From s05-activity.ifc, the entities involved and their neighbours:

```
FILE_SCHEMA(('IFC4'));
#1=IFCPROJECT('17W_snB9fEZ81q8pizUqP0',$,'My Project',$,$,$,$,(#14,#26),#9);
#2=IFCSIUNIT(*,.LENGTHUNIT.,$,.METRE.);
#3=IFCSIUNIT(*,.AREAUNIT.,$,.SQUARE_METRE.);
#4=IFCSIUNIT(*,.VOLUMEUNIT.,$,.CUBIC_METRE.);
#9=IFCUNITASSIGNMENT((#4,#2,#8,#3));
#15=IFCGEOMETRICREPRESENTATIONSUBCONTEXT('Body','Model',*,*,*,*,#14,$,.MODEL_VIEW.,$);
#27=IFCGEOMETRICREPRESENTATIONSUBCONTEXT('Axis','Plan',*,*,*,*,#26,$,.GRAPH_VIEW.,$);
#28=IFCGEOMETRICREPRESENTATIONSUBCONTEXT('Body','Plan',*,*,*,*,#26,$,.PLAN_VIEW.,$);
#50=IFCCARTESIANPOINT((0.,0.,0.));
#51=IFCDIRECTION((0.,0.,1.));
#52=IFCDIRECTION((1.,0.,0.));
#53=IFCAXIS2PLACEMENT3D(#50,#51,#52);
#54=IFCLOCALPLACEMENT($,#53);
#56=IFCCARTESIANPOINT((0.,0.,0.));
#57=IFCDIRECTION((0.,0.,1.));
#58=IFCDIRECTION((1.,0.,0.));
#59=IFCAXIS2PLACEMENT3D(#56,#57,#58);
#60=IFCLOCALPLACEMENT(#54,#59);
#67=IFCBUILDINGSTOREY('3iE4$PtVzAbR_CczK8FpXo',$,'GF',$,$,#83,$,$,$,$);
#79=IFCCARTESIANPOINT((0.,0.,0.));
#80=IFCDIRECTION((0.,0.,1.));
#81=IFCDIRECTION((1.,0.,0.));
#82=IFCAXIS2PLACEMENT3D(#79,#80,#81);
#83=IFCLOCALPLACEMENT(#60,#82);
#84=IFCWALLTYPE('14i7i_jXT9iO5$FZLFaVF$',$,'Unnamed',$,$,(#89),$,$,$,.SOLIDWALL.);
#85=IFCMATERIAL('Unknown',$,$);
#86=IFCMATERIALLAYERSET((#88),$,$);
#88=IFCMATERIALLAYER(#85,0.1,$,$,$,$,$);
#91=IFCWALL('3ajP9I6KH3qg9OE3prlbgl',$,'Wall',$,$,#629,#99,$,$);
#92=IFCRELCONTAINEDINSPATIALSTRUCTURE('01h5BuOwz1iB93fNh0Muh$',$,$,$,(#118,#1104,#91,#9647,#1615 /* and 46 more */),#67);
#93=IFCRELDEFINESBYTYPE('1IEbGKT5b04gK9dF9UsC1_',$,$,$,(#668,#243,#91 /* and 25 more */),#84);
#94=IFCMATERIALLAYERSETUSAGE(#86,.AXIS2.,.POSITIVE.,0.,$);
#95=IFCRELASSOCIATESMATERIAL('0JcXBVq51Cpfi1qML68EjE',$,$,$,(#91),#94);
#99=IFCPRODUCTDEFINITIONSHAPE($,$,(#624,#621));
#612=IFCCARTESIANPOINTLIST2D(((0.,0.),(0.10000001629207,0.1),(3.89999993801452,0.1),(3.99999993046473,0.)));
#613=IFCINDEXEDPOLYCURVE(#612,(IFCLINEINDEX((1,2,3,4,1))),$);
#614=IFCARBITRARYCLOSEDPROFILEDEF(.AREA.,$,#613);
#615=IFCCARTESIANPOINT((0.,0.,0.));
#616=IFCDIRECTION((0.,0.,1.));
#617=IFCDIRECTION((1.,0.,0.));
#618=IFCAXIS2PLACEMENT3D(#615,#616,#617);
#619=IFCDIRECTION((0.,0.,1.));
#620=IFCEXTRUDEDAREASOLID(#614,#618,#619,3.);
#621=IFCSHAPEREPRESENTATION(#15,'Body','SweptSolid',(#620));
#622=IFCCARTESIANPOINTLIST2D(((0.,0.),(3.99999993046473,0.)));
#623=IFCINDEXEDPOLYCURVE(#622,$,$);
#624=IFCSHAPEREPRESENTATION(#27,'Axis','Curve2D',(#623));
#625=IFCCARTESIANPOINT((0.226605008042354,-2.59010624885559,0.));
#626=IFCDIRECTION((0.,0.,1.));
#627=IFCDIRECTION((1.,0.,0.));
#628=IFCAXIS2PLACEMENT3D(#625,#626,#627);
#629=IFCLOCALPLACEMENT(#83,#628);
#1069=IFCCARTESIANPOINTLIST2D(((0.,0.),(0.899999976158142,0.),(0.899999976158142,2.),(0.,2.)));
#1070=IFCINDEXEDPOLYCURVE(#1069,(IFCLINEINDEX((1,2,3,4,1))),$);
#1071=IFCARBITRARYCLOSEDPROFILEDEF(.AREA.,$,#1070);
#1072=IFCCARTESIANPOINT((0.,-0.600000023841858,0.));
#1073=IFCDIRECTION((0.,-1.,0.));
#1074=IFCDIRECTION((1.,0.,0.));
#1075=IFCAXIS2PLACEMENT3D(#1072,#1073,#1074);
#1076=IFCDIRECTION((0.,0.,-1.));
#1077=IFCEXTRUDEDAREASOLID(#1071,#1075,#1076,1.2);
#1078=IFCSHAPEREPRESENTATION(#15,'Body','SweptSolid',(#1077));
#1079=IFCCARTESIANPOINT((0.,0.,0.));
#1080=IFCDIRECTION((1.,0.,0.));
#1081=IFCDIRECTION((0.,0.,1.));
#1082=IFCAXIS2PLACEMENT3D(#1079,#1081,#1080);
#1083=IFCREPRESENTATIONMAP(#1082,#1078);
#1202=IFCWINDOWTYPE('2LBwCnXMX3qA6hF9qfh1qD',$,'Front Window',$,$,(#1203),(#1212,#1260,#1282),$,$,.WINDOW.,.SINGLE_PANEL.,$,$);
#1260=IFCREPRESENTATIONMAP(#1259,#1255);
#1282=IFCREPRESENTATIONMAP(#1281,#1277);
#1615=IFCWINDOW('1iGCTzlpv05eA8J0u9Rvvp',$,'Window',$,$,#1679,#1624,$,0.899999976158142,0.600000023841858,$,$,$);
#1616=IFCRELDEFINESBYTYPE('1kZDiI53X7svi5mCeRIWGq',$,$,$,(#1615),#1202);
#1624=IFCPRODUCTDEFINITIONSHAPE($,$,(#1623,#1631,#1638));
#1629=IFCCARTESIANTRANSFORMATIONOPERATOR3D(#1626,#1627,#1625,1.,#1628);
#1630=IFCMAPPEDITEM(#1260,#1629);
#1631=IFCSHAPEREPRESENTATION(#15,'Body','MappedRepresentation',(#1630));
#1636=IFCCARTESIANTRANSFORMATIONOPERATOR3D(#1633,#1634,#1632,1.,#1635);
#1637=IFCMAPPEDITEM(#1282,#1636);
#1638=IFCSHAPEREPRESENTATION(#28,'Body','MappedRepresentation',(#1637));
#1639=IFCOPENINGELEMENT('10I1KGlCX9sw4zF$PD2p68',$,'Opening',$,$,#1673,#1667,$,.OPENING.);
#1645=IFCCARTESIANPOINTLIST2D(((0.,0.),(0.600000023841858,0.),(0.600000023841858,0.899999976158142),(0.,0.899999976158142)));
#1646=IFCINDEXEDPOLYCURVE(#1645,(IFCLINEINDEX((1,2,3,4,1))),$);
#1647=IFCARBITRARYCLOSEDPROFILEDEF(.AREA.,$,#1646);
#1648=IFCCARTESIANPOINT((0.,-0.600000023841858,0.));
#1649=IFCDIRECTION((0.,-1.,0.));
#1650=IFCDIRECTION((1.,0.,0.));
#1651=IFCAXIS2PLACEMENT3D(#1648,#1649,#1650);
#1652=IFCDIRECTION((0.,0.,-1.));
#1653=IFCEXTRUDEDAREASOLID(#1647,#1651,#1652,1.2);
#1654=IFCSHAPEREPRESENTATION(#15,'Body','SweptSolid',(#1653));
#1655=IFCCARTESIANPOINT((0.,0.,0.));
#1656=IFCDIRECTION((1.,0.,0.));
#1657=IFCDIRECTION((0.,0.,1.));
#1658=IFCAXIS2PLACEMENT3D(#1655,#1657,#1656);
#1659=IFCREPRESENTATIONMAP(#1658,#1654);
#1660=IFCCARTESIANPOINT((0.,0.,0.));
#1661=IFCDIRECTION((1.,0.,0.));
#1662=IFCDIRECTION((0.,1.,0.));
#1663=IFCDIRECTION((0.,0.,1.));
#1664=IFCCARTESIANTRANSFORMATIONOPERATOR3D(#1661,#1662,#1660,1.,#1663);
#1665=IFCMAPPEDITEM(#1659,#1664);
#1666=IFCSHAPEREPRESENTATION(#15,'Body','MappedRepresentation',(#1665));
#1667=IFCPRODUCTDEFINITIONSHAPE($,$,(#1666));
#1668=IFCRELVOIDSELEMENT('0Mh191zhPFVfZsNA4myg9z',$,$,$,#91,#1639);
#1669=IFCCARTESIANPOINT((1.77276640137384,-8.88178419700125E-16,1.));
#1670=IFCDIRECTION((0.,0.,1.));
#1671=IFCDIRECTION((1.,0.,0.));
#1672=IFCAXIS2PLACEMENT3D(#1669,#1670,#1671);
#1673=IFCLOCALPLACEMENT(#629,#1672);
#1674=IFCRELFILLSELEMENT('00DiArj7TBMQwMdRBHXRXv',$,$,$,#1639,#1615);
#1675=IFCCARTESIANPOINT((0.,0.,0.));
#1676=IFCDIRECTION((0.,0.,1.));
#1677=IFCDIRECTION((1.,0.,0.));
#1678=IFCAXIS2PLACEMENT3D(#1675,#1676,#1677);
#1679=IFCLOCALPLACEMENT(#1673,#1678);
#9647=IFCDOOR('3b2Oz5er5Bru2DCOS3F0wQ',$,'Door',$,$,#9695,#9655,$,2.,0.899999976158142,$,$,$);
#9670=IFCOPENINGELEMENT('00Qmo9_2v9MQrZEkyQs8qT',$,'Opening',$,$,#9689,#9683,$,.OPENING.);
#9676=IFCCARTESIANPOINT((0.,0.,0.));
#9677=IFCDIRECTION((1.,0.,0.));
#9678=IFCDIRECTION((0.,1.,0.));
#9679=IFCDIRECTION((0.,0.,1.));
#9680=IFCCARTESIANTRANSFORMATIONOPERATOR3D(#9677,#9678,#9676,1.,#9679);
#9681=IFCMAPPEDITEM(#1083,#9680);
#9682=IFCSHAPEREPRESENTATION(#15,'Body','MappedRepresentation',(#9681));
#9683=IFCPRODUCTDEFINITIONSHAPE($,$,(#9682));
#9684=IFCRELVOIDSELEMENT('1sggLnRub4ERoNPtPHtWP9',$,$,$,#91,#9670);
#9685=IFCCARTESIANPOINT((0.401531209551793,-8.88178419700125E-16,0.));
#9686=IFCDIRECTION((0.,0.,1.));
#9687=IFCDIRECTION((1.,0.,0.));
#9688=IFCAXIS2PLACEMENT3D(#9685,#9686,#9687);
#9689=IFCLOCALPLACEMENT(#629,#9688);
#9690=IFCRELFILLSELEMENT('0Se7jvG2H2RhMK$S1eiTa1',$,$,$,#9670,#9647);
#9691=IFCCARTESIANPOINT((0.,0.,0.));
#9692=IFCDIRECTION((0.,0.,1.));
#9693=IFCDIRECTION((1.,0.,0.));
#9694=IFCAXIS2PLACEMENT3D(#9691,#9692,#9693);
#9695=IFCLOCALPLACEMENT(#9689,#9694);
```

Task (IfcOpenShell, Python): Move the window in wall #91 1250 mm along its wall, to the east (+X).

```python
import ifcopenshell
import ifcopenshell.api.geometry
import ifcopenshell.util.placement
import ifcopenshell.util.unit

model = ifcopenshell.open("s05-activity.ifc")
unit_scale = ifcopenshell.util.unit.calculate_unit_scale(model)

window = model.by_id(1615)
opening = window.FillsVoids[0].RelatingOpeningElement
wall = opening.VoidsElements[0].RelatingBuildingElement

wall_matrix = ifcopenshell.util.placement.get_local_placement(wall.ObjectPlacement)
shift = wall_matrix[:3, 0] * 1.25 / unit_scale
before = ifcopenshell.util.placement.get_local_placement(window.ObjectPlacement)[:3, 3].copy()

# The window is placed relative to its opening, so it follows when the opening moves.
matrix = ifcopenshell.util.placement.get_local_placement(opening.ObjectPlacement)
matrix[:3, 3] += shift
ifcopenshell.api.geometry.edit_object_placement(
    model, product=opening, matrix=matrix, is_si=False, should_transform_children=True
)

after = ifcopenshell.util.placement.get_local_placement(window.ObjectPlacement)[:3, 3]
print("window moved by", (after - before).round(3) + 0.0)

model.write("s05-activity-out.ifc")
```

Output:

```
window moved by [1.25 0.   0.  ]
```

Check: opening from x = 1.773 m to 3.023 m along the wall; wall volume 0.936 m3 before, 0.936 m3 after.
